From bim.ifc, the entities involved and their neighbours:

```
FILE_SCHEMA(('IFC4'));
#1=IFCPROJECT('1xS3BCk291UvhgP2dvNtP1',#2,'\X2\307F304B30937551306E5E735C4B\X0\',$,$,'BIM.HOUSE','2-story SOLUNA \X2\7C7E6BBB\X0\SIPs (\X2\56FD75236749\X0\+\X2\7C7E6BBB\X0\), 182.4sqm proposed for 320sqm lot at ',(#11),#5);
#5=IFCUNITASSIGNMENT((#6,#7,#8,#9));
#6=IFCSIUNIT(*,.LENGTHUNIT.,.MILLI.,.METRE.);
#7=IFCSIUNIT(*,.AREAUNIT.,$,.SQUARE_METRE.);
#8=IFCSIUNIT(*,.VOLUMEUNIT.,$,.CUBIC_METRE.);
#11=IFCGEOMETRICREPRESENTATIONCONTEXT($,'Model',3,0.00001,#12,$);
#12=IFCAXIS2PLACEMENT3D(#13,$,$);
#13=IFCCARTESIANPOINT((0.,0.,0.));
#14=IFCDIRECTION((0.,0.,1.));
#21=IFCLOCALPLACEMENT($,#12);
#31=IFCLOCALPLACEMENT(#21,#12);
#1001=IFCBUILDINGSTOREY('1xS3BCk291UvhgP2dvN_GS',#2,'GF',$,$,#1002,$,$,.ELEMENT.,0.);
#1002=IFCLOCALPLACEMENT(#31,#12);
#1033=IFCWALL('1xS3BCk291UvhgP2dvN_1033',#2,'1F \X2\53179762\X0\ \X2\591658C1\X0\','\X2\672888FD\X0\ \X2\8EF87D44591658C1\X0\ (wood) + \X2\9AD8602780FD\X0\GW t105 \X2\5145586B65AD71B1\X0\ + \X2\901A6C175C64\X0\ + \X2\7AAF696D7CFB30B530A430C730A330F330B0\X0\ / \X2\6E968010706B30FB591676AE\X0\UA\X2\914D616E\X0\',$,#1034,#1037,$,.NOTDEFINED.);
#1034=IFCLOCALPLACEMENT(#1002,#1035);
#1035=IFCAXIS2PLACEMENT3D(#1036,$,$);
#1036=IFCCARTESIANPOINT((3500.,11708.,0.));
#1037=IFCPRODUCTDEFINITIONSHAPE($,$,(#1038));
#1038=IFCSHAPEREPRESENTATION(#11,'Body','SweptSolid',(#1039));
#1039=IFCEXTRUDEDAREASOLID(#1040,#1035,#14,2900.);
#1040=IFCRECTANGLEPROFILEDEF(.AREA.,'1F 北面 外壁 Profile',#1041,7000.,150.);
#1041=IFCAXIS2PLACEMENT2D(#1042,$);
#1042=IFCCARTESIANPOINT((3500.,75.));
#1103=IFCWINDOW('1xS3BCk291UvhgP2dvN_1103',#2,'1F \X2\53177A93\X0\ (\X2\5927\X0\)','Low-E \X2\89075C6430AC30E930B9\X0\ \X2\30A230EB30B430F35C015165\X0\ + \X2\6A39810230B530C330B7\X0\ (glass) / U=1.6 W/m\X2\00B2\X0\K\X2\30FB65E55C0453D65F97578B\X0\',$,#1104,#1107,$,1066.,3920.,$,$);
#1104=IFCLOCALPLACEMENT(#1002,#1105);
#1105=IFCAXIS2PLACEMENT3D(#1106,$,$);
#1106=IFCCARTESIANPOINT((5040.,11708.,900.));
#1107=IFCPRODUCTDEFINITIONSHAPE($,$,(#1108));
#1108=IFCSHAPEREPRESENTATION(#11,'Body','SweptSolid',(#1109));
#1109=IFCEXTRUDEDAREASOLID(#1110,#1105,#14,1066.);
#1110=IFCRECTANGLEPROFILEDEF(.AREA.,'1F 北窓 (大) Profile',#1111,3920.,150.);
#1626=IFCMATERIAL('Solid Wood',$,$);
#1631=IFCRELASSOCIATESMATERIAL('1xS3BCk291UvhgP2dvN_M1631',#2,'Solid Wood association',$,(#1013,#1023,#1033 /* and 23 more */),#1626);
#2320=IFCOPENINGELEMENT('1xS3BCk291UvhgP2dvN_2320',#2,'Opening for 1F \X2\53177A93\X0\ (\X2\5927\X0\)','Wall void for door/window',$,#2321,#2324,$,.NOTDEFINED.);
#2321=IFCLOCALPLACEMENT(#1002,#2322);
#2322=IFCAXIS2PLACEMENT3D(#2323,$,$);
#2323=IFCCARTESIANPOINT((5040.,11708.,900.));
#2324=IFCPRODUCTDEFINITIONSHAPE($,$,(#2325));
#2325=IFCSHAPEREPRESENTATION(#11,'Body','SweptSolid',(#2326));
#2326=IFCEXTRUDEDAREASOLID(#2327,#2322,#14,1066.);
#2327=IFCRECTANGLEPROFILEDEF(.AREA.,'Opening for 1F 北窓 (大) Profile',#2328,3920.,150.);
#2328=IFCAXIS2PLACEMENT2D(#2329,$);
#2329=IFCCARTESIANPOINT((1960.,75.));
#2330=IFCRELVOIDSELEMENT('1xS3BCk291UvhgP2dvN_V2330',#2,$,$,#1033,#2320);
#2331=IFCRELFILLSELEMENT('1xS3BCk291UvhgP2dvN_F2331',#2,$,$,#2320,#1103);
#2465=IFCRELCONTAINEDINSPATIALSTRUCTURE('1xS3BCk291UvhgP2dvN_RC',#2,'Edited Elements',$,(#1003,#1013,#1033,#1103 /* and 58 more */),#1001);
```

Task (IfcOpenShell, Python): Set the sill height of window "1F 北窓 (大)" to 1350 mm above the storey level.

```python
import numpy as np
import ifcopenshell
import ifcopenshell.api.geometry
import ifcopenshell.geom
import ifcopenshell.util.element
import ifcopenshell.util.placement
import ifcopenshell.util.shape
import ifcopenshell.util.unit

model = ifcopenshell.open("bim.ifc")
unit_scale = ifcopenshell.util.unit.calculate_unit_scale(model)

window = model.by_id(1103)
opening = window.FillsVoids[0].RelatingOpeningElement
storey = ifcopenshell.util.element.get_container(window, ifc_class="IfcBuildingStorey")
level = ifcopenshell.util.placement.get_local_placement(storey.ObjectPlacement)[2, 3]

# The opening's origin need not be at the sill, so measure its lowest point.
shape = ifcopenshell.geom.create_shape(ifcopenshell.geom.settings(), opening)
bottom = ifcopenshell.util.shape.get_shape_bottom_elevation(shape, shape.geometry) / unit_scale
dz = level + 1.35 / unit_scale - bottom

shift = np.array([0.0, 0.0, dz])
# The window is not placed relative to its opening, so move both.
for product in (opening, window):
    matrix = ifcopenshell.util.placement.get_local_placement(product.ObjectPlacement)
    matrix[:3, 3] += shift
    ifcopenshell.api.geometry.edit_object_placement(model, product=product, matrix=matrix, is_si=False)

print(f"moved by {dz * unit_scale:+.3f} m")

model.write("bim_rev.ifc")
```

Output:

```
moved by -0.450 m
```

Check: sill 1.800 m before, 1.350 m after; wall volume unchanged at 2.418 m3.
